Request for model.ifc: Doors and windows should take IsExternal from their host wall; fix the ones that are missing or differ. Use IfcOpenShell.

First a look at what the model holds.

```python
import ifcopenshell
import ifcopenshell.util.element

model = ifcopenshell.open("model.ifc")
print(model.schema)
seen = {}
for e in model.by_type("IfcDoor") + model.by_type("IfcWindow"):
    if not e.FillsVoids:
        continue
    host = e.FillsVoids[0].RelatingOpeningElement.VoidsElements[0].RelatingBuildingElement
    own = ifcopenshell.util.element.get_pset(e, f"Pset_{e.is_a()[3:].removesuffix('StandardCase')}Common", "IsExternal")
    wall = ifcopenshell.util.element.get_pset(host, "Pset_WallCommon", "IsExternal")
    seen[e.is_a(), own, wall] = seen.get((e.is_a(), own, wall), 0) + 1
for (cls, own, wall), count in sorted(seen.items(), key=str):
    print(count, cls, "IsExternal:", own, "| host wall:", wall)
```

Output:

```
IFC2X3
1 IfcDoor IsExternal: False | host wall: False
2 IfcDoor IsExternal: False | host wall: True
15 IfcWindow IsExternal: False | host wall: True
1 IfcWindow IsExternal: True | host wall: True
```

```python
import ifcopenshell
import ifcopenshell.api.pset
import ifcopenshell.util.element

model = ifcopenshell.open("model.ifc")

count = 0
for ifc_class, pset_name in (("IfcDoor", "Pset_DoorCommon"), ("IfcWindow", "Pset_WindowCommon")):
    for e in model.by_type(ifc_class):
        if not e.FillsVoids:
            continue
        host = e.FillsVoids[0].RelatingOpeningElement.VoidsElements[0].RelatingBuildingElement
        external = ifcopenshell.util.element.get_pset(host, "Pset_WallCommon", "IsExternal")
        if external is None or ifcopenshell.util.element.get_pset(e, pset_name, "IsExternal") == external:
            continue
        pset = ifcopenshell.api.pset.add_pset(model, product=e, name=pset_name)
        ifcopenshell.api.pset.edit_pset(model, pset=pset, properties={"IsExternal": external})
        count += 1

print(count, "updated")

model.write("model_v2.ifc")
```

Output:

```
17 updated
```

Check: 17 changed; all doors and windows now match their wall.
